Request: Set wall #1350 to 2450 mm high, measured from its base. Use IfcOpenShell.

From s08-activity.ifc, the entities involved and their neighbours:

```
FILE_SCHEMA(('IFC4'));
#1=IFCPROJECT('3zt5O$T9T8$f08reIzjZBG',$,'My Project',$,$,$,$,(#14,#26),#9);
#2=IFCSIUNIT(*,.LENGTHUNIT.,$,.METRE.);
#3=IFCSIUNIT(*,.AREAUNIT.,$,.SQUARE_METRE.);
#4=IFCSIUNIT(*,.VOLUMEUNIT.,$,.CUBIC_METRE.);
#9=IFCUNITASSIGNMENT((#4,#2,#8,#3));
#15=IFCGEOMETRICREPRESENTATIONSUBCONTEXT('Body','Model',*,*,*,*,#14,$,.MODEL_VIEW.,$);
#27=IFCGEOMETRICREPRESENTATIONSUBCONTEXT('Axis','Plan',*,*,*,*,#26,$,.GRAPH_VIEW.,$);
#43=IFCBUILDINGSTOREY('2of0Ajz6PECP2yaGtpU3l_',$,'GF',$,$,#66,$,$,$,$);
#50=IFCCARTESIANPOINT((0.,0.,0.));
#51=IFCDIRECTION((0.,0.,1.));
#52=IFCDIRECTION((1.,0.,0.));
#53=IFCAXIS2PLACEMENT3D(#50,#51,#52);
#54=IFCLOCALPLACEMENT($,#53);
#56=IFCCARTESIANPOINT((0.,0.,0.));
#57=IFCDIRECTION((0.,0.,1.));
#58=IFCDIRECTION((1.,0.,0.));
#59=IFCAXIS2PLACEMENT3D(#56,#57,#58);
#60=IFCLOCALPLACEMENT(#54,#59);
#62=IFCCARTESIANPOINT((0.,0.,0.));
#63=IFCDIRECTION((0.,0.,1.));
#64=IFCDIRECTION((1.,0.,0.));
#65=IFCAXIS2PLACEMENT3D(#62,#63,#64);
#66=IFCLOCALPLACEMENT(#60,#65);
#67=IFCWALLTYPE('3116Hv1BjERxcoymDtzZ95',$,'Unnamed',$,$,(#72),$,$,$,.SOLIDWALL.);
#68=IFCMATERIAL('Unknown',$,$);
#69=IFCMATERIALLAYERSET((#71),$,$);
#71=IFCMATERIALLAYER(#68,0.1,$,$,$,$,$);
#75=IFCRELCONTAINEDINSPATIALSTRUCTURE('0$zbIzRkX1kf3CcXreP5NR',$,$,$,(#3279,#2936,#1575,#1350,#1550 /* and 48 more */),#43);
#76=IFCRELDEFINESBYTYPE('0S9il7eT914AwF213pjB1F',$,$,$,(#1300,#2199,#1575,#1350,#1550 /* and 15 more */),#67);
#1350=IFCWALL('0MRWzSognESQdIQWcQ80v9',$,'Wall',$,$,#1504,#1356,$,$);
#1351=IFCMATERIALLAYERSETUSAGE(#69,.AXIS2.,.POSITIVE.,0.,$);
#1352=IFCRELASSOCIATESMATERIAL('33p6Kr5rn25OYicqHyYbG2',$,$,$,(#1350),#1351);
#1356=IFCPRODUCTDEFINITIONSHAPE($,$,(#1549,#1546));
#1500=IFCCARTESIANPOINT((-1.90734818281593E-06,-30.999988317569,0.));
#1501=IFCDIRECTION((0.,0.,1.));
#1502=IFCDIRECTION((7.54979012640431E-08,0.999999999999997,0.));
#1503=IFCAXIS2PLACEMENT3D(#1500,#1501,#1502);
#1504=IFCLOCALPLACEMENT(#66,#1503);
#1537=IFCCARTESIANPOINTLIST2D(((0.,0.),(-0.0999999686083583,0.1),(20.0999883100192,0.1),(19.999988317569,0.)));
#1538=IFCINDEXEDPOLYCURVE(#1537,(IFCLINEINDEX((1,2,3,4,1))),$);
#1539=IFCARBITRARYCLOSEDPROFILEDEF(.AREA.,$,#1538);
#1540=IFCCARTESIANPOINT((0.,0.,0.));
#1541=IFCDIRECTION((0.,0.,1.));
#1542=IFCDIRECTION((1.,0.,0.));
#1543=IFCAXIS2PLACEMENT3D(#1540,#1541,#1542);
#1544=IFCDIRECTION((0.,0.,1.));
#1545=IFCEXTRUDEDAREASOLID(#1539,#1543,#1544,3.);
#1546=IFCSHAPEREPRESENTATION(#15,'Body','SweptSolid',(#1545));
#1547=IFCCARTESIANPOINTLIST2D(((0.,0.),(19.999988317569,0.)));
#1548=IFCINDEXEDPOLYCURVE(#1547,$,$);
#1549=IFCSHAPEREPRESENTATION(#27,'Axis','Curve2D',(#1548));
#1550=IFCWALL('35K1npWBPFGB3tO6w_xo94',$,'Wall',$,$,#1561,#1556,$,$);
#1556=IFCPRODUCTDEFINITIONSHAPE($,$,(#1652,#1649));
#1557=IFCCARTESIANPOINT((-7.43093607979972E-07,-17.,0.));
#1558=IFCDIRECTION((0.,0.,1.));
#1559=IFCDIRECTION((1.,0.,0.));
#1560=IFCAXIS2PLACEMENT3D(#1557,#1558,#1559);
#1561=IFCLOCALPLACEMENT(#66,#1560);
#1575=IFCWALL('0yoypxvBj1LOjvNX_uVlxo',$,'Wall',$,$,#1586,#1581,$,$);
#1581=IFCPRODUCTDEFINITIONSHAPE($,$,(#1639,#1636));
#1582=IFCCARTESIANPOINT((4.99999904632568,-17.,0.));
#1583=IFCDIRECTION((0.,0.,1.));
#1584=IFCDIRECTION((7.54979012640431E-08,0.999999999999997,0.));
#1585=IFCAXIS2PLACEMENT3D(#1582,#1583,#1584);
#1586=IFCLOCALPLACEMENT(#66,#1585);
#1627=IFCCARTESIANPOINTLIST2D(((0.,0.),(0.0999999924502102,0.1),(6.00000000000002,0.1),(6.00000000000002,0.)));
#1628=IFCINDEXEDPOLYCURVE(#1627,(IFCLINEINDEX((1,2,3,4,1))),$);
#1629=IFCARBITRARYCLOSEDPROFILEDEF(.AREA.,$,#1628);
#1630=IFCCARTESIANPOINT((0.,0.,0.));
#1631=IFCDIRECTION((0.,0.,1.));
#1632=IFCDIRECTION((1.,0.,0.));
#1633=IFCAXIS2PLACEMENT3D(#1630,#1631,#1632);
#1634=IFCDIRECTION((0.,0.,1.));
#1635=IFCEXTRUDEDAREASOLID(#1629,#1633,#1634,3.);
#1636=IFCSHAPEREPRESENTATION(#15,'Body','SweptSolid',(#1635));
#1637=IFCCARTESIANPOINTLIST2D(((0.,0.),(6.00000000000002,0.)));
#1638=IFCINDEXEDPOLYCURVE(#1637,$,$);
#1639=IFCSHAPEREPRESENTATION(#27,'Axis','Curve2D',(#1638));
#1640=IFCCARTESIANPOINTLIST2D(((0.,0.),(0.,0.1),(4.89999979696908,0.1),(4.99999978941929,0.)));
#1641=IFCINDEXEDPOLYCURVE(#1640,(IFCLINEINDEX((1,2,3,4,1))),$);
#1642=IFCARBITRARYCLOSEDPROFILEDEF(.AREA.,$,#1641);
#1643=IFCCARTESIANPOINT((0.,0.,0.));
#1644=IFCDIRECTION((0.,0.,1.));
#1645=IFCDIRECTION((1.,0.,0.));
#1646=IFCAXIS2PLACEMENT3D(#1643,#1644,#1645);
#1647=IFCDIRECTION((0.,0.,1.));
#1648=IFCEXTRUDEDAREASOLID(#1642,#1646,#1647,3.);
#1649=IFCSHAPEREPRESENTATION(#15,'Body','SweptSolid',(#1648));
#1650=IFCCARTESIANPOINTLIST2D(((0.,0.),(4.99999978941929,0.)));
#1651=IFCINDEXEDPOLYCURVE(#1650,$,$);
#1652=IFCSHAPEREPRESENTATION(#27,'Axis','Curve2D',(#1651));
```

```python
import ifcopenshell
import ifcopenshell.geom
import ifcopenshell.util.representation
import ifcopenshell.util.shape

model = ifcopenshell.open("s08-activity.ifc")
settings = ifcopenshell.geom.settings()


def volume(element):
    """Net volume in cubic metres, openings subtracted."""
    shape = ifcopenshell.geom.create_shape(settings, element)
    return ifcopenshell.util.shape.get_volume(shape.geometry)


wall = model.by_id(1350)
before = volume(wall)

body = ifcopenshell.util.representation.get_representation(wall, "Model", "Body")
solid = body.Items[0]
old_height = solid.Depth
solid.Depth = 2.45
after = volume(wall)

print(f"height {old_height:g} -> {solid.Depth:g}, volume {before:.3f} -> {after:.3f} m3")

model.write("s08-activity_v2.ifc")
```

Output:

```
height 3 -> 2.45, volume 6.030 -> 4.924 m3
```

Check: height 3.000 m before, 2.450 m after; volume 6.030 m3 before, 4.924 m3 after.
